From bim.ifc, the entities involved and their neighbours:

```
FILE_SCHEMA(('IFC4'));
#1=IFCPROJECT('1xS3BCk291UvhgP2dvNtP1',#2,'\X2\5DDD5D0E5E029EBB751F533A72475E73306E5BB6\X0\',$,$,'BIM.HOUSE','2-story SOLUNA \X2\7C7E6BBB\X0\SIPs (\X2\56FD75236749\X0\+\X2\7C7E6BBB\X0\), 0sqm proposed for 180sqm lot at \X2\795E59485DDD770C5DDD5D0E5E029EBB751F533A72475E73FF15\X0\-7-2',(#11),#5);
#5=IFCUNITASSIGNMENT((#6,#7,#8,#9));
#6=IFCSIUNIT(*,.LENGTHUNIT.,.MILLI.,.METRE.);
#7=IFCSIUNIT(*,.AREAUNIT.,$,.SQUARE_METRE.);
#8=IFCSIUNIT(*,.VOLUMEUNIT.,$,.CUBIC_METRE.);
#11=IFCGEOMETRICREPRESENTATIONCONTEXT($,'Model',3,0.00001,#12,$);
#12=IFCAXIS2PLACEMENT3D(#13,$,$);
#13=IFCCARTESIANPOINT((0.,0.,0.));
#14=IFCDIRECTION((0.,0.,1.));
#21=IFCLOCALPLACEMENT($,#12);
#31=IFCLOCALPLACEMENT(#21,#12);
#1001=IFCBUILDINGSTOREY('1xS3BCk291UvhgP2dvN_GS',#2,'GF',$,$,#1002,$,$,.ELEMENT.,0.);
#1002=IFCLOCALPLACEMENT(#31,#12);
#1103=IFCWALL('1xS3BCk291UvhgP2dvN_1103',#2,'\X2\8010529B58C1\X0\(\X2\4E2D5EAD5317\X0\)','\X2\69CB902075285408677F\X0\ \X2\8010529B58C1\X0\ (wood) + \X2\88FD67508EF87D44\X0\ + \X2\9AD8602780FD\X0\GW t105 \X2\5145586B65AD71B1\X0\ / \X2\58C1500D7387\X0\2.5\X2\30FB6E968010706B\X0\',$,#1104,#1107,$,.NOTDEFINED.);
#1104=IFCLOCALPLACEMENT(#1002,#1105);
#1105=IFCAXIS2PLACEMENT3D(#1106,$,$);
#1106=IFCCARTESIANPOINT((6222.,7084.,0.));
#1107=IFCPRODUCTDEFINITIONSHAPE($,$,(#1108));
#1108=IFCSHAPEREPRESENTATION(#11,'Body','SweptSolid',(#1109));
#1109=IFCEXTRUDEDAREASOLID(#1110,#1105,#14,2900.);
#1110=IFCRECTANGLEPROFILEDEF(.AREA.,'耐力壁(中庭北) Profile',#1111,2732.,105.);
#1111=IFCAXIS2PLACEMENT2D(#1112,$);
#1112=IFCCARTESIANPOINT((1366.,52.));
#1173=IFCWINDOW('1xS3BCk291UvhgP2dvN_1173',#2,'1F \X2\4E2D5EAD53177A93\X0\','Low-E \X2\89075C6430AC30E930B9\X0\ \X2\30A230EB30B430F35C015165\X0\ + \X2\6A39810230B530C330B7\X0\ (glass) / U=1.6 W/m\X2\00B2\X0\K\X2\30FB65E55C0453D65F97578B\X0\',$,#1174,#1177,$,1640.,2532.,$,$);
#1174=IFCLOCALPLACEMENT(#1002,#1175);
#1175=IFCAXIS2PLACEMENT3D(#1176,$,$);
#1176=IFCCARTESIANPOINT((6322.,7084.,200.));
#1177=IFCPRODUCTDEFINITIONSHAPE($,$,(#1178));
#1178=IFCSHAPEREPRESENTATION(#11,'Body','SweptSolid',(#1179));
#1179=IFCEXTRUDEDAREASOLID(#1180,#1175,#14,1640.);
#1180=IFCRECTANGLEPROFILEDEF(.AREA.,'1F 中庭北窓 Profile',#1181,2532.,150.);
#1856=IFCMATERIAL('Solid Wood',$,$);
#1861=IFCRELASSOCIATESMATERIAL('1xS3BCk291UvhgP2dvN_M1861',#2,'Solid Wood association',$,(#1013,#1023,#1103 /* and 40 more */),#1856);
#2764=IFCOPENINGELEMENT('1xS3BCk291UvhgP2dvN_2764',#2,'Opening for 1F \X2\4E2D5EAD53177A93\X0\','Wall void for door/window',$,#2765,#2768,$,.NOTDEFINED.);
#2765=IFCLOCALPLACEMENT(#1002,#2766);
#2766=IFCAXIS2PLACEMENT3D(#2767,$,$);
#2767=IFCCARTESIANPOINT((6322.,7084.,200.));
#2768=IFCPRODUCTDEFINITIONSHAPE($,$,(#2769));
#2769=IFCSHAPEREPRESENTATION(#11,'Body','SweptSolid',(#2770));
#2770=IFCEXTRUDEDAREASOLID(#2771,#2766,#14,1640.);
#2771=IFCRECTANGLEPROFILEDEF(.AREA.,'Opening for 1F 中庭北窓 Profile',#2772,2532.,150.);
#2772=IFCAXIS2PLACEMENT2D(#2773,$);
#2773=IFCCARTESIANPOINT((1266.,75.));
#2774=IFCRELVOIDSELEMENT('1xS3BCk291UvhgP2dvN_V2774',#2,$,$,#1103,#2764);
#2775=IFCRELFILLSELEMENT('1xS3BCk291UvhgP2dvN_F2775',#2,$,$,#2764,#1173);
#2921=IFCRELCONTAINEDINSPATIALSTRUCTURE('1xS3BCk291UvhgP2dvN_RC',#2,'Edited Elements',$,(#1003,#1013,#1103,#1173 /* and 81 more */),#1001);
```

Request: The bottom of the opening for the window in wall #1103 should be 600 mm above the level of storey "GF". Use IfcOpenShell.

```python
import numpy as np
import ifcopenshell
import ifcopenshell.api.geometry
import ifcopenshell.geom
import ifcopenshell.util.element
import ifcopenshell.util.placement
import ifcopenshell.util.shape
import ifcopenshell.util.unit

model = ifcopenshell.open("bim.ifc")
unit_scale = ifcopenshell.util.unit.calculate_unit_scale(model)

window = model.by_id(1173)
opening = window.FillsVoids[0].RelatingOpeningElement
storey = ifcopenshell.util.element.get_container(window, ifc_class="IfcBuildingStorey")
level = ifcopenshell.util.placement.get_local_placement(storey.ObjectPlacement)[2, 3]

# The opening's origin need not be at the sill, so measure its lowest point.
shape = ifcopenshell.geom.create_shape(ifcopenshell.geom.settings(), opening)
bottom = ifcopenshell.util.shape.get_shape_bottom_elevation(shape, shape.geometry) / unit_scale
dz = level + 600.0 - bottom

shift = np.array([0.0, 0.0, dz])
# The window is not placed relative to its opening, so move both.
for product in (opening, window):
    matrix = ifcopenshell.util.placement.get_local_placement(product.ObjectPlacement)
    matrix[:3, 3] += shift
    ifcopenshell.api.geometry.edit_object_placement(model, product=product, matrix=matrix, is_si=False)

print(f"moved by {dz * unit_scale:+.3f} m")

model.write("bim_updated.ifc")
```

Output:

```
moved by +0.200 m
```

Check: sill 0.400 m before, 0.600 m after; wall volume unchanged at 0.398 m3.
